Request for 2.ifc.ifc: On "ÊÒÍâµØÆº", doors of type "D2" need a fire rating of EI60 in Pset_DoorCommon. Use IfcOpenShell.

First a look at what the model holds.

```python
import ifcopenshell
import ifcopenshell.util.element

model = ifcopenshell.open("2.ifc.ifc")
print(model.schema)
storey = next(s for s in model.by_type("IfcBuildingStorey") if s.Name == "ÊÒÍâµØÆº")
doors = [e for e in ifcopenshell.util.element.get_decomposition(storey) if e.is_a("IfcDoor")]
seen = {}
for e in doors:
    element_type = ifcopenshell.util.element.get_type(e)
    key = (element_type.Name if element_type != e and element_type else None, ifcopenshell.util.element.get_pset(e, "Pset_DoorCommon", "FireRating"))
    seen[key] = seen.get(key, 0) + 1
for (name, value), count in sorted(seen.items(), key=str):
    print(count, "x", name, "|", value)
```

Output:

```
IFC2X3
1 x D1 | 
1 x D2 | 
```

```python
import ifcopenshell
import ifcopenshell.api.pset
import ifcopenshell.util.element

model = ifcopenshell.open("2.ifc.ifc")

storey = next(s for s in model.by_type("IfcBuildingStorey") if s.Name == "ÊÒÍâµØÆº")
doors = [e for e in ifcopenshell.util.element.get_decomposition(storey) if e.is_a("IfcDoor")]

count = 0
for e in doors:
    element_type = ifcopenshell.util.element.get_type(e)
    if element_type in (None, e) or element_type.Name != "D2":
        continue
    # add_pset returns the element's existing set when there is one.
    pset = ifcopenshell.api.pset.add_pset(model, product=e, name="Pset_DoorCommon")
    ifcopenshell.api.pset.edit_pset(model, pset=pset, properties={"FireRating": "EI60"})
    count += 1

print(count, "doors updated")

model.write("2.ifc_rev.ifc")
```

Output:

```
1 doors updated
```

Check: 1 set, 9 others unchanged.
